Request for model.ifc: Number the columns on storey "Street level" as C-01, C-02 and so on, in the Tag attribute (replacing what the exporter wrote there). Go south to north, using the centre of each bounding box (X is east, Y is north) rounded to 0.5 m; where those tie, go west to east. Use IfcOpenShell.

First a look at what the model holds.

```python
import ifcopenshell
import ifcopenshell.util.element
import ifcopenshell.util.placement

model = ifcopenshell.open("model.ifc")
print(model.schema)
storey = next(s for s in model.by_type("IfcBuildingStorey") if s.Name == "Street level")
columns = [e for e in ifcopenshell.util.element.get_decomposition(storey) if e.is_a("IfcColumn")]
for e in sorted(columns, key=lambda e: e.id()):
    origin = ifcopenshell.util.placement.get_local_placement(e.ObjectPlacement)[:3, 3]
    print(e.id(), e.Tag, e.Name, origin.round(2) + 0.0, sep=" | ")
```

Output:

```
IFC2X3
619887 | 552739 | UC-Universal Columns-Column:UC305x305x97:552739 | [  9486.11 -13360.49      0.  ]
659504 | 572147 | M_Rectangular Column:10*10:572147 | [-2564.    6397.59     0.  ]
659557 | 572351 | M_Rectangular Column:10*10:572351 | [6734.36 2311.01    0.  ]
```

```python
import ifcopenshell
import ifcopenshell.geom
import ifcopenshell.util.element
import ifcopenshell.util.shape

model = ifcopenshell.open("model.ifc")
settings = ifcopenshell.geom.settings()
settings.set("use-world-coords", True)


def centre(element):
    shape = ifcopenshell.geom.create_shape(settings, element)
    return ifcopenshell.util.shape.get_bbox_centroid(shape.geometry)


storey = next(s for s in model.by_type("IfcBuildingStorey") if s.Name == "Street level")
columns = [e for e in ifcopenshell.util.element.get_decomposition(storey) if e.is_a("IfcColumn")]

# Insertion points can sit at a corner or the storey origin, so sort by the geometry (in metres).
centres = {e: centre(e) for e in columns}
columns.sort(key=lambda e: (round(centres[e][1] / 0.5), centres[e][0]))

for i, e in enumerate(columns, start=1):
    number = f"C-{i:02d}"
    e.Tag = number
    print(e.id(), number)

model.write("model-out.ifc")
```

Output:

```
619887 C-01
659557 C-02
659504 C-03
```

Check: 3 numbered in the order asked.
